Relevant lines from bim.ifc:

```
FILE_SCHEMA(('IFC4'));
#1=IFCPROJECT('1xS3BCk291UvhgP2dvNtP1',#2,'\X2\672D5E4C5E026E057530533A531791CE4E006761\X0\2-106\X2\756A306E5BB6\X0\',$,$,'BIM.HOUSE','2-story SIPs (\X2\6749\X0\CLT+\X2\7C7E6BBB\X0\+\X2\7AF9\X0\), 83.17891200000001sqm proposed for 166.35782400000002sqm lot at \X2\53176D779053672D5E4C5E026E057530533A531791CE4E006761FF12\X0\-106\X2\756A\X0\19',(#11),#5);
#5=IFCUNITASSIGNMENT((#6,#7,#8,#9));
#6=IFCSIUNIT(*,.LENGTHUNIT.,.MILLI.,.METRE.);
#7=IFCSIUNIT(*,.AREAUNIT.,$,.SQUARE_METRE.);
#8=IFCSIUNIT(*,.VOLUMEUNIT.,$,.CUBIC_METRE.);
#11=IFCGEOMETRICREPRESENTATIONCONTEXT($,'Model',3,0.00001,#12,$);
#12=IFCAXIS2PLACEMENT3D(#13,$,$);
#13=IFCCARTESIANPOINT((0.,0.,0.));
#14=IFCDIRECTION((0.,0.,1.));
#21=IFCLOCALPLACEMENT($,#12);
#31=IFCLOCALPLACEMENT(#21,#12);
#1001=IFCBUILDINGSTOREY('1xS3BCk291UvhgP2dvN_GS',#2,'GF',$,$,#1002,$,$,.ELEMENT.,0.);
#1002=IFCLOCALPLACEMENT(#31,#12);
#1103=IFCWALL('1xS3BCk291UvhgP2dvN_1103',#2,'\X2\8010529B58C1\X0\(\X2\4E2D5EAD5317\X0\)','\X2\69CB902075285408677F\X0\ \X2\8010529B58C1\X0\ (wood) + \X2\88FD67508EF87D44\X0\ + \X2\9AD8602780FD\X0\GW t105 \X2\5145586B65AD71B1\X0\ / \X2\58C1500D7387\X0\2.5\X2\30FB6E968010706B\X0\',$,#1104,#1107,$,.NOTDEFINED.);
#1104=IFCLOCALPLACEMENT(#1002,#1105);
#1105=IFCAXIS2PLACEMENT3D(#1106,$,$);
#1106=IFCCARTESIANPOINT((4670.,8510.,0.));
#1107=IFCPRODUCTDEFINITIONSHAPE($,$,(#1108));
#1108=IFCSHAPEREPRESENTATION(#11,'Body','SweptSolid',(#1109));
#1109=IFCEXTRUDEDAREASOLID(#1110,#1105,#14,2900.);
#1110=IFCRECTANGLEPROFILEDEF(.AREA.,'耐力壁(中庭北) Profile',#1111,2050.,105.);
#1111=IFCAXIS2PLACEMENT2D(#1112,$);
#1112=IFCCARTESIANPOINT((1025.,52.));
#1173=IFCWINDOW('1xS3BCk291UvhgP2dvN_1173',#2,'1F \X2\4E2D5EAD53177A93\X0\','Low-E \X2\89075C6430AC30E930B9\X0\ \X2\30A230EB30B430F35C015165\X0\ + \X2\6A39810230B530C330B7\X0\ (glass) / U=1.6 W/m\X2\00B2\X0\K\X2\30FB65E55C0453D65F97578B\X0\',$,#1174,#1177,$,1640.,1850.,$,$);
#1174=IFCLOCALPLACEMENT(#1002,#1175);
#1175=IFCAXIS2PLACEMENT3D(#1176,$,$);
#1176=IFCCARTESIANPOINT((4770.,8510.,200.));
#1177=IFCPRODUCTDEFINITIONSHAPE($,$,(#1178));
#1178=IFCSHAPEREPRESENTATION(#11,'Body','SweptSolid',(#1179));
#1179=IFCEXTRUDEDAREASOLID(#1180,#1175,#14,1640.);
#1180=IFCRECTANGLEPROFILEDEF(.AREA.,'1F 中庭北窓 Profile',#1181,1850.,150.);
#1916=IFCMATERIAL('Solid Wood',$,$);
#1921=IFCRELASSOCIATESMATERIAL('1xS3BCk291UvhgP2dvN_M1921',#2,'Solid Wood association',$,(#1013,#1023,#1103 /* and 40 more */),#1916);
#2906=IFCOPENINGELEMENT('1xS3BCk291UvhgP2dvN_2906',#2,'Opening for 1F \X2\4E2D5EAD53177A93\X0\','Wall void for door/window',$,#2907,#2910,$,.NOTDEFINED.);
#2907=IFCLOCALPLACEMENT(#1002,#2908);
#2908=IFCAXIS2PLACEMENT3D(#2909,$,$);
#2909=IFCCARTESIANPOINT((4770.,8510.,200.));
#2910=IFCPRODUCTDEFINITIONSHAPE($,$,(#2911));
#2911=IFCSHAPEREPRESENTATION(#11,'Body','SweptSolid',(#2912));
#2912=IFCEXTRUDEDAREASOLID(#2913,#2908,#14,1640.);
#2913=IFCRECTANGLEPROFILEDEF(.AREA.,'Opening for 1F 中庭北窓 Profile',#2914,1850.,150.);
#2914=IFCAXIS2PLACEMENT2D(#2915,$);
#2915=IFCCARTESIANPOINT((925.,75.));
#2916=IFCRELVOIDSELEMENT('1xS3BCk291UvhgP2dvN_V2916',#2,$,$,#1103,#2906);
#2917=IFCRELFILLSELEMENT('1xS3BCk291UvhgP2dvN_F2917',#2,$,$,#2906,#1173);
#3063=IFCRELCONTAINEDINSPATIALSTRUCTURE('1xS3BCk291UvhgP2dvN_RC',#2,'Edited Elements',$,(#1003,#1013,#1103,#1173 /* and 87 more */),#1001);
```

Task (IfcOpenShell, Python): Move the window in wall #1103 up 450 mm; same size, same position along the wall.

```python
import numpy as np
import ifcopenshell
import ifcopenshell.api.geometry
import ifcopenshell.util.placement
import ifcopenshell.util.unit

model = ifcopenshell.open("bim.ifc")
unit_scale = ifcopenshell.util.unit.calculate_unit_scale(model)

window = model.by_guid("1xS3BCk291UvhgP2dvN_1173")
opening = window.FillsVoids[0].RelatingOpeningElement
dz = 450.0

shift = np.array([0.0, 0.0, dz])
# The window is not placed relative to its opening, so move both.
for product in (opening, window):
    matrix = ifcopenshell.util.placement.get_local_placement(product.ObjectPlacement)
    matrix[:3, 3] += shift
    ifcopenshell.api.geometry.edit_object_placement(model, product=product, matrix=matrix, is_si=False)

print(f"moved by {dz * unit_scale:+.3f} m")

model.write("bim_v2.ifc")
```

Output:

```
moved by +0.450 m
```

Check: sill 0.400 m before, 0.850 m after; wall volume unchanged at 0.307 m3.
